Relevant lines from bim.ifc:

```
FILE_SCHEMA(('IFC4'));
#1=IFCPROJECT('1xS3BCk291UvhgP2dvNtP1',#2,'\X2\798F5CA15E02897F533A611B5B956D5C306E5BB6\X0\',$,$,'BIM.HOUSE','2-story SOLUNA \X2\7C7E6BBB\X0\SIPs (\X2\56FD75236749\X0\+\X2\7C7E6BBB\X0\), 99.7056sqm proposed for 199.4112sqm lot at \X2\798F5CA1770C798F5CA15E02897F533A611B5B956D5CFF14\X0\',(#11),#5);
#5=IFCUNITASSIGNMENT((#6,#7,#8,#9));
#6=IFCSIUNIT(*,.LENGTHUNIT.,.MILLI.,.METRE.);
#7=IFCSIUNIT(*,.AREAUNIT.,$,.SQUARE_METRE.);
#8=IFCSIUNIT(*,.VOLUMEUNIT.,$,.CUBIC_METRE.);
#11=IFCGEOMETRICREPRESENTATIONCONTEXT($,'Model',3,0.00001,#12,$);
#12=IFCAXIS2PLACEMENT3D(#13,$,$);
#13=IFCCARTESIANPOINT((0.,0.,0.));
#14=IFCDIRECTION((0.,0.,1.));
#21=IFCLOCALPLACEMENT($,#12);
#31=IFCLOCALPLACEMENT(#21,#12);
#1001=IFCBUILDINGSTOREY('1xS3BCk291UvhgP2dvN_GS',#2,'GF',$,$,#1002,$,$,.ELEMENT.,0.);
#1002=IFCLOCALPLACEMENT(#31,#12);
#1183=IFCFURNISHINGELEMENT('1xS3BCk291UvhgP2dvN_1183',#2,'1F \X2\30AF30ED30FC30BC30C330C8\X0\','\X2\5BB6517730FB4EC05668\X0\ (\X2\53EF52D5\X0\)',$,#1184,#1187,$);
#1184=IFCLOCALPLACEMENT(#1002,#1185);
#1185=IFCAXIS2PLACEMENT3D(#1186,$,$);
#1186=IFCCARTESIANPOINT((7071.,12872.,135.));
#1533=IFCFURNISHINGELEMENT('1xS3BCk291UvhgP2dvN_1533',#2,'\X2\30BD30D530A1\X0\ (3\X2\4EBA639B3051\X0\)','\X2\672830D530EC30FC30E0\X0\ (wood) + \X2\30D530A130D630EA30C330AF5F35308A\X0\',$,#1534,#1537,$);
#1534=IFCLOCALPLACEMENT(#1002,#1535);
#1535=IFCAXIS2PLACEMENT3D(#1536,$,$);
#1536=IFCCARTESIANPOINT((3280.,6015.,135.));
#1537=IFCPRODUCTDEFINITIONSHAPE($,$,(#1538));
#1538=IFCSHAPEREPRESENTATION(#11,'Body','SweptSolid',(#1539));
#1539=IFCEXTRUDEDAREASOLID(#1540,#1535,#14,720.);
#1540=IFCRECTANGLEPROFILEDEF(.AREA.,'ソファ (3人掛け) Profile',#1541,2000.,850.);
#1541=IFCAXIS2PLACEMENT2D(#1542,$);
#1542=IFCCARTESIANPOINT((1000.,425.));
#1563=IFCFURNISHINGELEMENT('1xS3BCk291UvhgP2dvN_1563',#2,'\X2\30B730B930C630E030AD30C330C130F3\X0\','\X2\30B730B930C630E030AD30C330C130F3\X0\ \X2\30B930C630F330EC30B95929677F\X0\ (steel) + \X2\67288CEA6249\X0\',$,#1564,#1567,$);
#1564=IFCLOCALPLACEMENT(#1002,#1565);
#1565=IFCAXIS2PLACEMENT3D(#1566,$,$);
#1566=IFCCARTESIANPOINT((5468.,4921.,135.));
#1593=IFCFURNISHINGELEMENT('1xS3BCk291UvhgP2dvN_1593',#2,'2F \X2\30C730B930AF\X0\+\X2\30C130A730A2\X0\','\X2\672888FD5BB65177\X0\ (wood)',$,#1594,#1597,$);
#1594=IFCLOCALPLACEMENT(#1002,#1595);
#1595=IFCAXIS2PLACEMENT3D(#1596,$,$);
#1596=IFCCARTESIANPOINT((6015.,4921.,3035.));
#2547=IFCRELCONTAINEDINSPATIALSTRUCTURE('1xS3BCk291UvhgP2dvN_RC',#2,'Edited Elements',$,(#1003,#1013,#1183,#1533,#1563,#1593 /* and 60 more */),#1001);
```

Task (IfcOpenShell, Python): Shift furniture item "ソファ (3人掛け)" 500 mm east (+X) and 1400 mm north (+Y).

```python
import ifcopenshell
import ifcopenshell.api.geometry
import ifcopenshell.util.placement

model = ifcopenshell.open("bim.ifc")

item = model.by_guid("1xS3BCk291UvhgP2dvN_1533")
matrix = ifcopenshell.util.placement.get_local_placement(item.ObjectPlacement)
matrix[0, 3] += 500.0
matrix[1, 3] += 1400.0
ifcopenshell.api.geometry.edit_object_placement(model, product=item, matrix=matrix, is_si=False)

print(ifcopenshell.util.placement.get_local_placement(item.ObjectPlacement).round(3) + 0.0)

model.write("bim_rev.ifc")
```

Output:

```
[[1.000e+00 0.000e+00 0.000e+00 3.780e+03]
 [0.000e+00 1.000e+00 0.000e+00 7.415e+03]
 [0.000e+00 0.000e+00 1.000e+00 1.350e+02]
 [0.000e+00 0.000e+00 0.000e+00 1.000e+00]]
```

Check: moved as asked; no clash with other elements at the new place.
